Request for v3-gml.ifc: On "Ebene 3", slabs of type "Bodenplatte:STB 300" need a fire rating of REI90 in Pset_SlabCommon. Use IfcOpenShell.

First a look at what the model holds.

```python
import ifcopenshell
import ifcopenshell.util.element

model = ifcopenshell.open("v3-gml.ifc")
print(model.schema)
storey = next(s for s in model.by_type("IfcBuildingStorey") if s.Name == "Ebene 3")
slabs = [e for e in ifcopenshell.util.element.get_decomposition(storey) if e.is_a("IfcSlab")]
seen = {}
for e in slabs:
    element_type = ifcopenshell.util.element.get_type(e)
    key = (element_type.Name if element_type != e and element_type else None, ifcopenshell.util.element.get_pset(e, "Pset_SlabCommon", "FireRating"))
    seen[key] = seen.get(key, 0) + 1
for (name, value), count in sorted(seen.items(), key=str):
    print(count, "x", name, "|", value)
```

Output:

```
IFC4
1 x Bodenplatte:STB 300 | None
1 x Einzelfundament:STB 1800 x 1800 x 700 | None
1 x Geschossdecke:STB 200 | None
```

```python
import ifcopenshell
import ifcopenshell.api.pset
import ifcopenshell.util.element

model = ifcopenshell.open("v3-gml.ifc")

storey = next(s for s in model.by_type("IfcBuildingStorey") if s.Name == "Ebene 3")
slabs = [e for e in ifcopenshell.util.element.get_decomposition(storey) if e.is_a("IfcSlab")]

count = 0
for e in slabs:
    element_type = ifcopenshell.util.element.get_type(e)
    if element_type in (None, e) or element_type.Name != "Bodenplatte:STB 300":
        continue
    # add_pset returns the element's existing set when there is one.
    pset = ifcopenshell.api.pset.add_pset(model, product=e, name="Pset_SlabCommon")
    ifcopenshell.api.pset.edit_pset(model, pset=pset, properties={"FireRating": "REI90"})
    count += 1

print(count, "slabs updated")

model.write("v3-gml_edited.ifc")
```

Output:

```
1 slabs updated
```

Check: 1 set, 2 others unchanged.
